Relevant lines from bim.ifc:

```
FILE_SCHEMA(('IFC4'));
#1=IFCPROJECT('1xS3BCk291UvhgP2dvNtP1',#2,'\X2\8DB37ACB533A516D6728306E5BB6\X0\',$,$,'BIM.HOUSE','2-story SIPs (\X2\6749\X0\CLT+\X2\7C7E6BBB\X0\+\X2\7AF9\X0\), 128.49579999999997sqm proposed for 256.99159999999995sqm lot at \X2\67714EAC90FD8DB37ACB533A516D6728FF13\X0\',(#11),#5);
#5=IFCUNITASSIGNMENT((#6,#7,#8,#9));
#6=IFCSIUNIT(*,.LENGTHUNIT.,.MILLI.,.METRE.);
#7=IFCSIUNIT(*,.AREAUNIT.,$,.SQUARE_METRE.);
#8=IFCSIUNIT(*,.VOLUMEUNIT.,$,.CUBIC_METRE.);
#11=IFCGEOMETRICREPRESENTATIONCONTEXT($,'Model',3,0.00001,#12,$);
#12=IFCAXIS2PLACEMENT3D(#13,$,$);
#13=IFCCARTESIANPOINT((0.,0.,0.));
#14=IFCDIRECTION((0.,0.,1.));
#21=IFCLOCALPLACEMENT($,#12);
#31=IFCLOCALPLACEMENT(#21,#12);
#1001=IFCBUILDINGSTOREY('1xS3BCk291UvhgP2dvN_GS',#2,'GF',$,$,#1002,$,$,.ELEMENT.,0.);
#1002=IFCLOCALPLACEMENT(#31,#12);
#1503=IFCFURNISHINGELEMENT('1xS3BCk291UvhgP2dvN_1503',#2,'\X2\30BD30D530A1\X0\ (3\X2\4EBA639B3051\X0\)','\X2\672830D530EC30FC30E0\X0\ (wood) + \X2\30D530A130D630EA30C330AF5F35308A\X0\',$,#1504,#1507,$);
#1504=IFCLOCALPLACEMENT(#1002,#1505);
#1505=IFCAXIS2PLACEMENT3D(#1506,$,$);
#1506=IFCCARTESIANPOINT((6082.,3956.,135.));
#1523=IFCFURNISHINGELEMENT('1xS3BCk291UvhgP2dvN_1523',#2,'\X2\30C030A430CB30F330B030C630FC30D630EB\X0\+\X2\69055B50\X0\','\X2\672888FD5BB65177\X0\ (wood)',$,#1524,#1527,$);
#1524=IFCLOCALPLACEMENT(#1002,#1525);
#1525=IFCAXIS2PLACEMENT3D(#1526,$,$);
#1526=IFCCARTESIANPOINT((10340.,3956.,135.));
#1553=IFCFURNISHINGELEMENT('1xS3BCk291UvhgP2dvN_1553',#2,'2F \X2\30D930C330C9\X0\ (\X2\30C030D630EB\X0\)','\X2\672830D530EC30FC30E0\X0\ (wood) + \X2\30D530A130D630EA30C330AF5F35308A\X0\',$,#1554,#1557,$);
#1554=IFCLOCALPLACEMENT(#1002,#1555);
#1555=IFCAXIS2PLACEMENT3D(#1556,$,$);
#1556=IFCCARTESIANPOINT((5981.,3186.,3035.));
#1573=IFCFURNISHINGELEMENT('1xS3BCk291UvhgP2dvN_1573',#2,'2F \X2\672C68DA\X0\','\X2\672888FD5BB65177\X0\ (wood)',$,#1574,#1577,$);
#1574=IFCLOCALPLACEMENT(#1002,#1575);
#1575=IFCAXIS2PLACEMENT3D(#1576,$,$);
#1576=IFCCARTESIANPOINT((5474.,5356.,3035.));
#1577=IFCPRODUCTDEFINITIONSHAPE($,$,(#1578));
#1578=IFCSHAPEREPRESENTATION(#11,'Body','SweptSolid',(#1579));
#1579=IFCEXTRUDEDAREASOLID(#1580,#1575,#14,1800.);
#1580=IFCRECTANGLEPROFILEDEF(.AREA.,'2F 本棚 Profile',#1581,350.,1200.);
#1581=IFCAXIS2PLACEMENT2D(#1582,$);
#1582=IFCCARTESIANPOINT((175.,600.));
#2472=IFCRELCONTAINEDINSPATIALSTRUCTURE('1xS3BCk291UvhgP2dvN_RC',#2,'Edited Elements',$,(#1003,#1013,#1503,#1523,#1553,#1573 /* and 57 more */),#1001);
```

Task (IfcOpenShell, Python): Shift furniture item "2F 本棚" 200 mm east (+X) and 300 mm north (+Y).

```python
import ifcopenshell
import ifcopenshell.api.geometry
import ifcopenshell.util.placement

model = ifcopenshell.open("bim.ifc")

item = model.by_guid("1xS3BCk291UvhgP2dvN_1573")
matrix = ifcopenshell.util.placement.get_local_placement(item.ObjectPlacement)
matrix[0, 3] += 200.0
matrix[1, 3] += 300.0
ifcopenshell.api.geometry.edit_object_placement(model, product=item, matrix=matrix, is_si=False)

print(ifcopenshell.util.placement.get_local_placement(item.ObjectPlacement).round(3) + 0.0)

model.write("bim_v2.ifc")
```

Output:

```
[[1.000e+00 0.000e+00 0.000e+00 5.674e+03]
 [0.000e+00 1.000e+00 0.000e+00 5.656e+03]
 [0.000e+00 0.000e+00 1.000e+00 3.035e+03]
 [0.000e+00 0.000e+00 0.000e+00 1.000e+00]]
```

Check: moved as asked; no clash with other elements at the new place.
